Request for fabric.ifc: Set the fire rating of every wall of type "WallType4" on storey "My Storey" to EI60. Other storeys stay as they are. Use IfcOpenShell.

First a look at what the model holds.

```python
import ifcopenshell
import ifcopenshell.util.element

model = ifcopenshell.open("fabric.ifc")
print(model.schema)
storey = next(s for s in model.by_type("IfcBuildingStorey") if s.Name == "My Storey")
walls = [e for e in ifcopenshell.util.element.get_decomposition(storey) if e.is_a("IfcWall")]
seen = {}
for e in walls:
    element_type = ifcopenshell.util.element.get_type(e)
    key = (element_type.Name if element_type != e and element_type else None, ifcopenshell.util.element.get_pset(e, "Pset_WallCommon", "FireRating"))
    seen[key] = seen.get(key, 0) + 1
for (name, value), count in sorted(seen.items(), key=str):
    print(count, "x", name, "|", value)
```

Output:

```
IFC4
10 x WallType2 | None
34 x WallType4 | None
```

```python
import ifcopenshell
import ifcopenshell.api.pset
import ifcopenshell.util.element

model = ifcopenshell.open("fabric.ifc")

storey = next(s for s in model.by_type("IfcBuildingStorey") if s.Name == "My Storey")
walls = [e for e in ifcopenshell.util.element.get_decomposition(storey) if e.is_a("IfcWall")]

count = 0
for e in walls:
    element_type = ifcopenshell.util.element.get_type(e)
    if element_type in (None, e) or element_type.Name != "WallType4":
        continue
    # add_pset returns the element's existing set when there is one.
    pset = ifcopenshell.api.pset.add_pset(model, product=e, name="Pset_WallCommon")
    ifcopenshell.api.pset.edit_pset(model, pset=pset, properties={"FireRating": "EI60"})
    count += 1

print(count, "walls updated")

model.write("fabric_edited.ifc")
```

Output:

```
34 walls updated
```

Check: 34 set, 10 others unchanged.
